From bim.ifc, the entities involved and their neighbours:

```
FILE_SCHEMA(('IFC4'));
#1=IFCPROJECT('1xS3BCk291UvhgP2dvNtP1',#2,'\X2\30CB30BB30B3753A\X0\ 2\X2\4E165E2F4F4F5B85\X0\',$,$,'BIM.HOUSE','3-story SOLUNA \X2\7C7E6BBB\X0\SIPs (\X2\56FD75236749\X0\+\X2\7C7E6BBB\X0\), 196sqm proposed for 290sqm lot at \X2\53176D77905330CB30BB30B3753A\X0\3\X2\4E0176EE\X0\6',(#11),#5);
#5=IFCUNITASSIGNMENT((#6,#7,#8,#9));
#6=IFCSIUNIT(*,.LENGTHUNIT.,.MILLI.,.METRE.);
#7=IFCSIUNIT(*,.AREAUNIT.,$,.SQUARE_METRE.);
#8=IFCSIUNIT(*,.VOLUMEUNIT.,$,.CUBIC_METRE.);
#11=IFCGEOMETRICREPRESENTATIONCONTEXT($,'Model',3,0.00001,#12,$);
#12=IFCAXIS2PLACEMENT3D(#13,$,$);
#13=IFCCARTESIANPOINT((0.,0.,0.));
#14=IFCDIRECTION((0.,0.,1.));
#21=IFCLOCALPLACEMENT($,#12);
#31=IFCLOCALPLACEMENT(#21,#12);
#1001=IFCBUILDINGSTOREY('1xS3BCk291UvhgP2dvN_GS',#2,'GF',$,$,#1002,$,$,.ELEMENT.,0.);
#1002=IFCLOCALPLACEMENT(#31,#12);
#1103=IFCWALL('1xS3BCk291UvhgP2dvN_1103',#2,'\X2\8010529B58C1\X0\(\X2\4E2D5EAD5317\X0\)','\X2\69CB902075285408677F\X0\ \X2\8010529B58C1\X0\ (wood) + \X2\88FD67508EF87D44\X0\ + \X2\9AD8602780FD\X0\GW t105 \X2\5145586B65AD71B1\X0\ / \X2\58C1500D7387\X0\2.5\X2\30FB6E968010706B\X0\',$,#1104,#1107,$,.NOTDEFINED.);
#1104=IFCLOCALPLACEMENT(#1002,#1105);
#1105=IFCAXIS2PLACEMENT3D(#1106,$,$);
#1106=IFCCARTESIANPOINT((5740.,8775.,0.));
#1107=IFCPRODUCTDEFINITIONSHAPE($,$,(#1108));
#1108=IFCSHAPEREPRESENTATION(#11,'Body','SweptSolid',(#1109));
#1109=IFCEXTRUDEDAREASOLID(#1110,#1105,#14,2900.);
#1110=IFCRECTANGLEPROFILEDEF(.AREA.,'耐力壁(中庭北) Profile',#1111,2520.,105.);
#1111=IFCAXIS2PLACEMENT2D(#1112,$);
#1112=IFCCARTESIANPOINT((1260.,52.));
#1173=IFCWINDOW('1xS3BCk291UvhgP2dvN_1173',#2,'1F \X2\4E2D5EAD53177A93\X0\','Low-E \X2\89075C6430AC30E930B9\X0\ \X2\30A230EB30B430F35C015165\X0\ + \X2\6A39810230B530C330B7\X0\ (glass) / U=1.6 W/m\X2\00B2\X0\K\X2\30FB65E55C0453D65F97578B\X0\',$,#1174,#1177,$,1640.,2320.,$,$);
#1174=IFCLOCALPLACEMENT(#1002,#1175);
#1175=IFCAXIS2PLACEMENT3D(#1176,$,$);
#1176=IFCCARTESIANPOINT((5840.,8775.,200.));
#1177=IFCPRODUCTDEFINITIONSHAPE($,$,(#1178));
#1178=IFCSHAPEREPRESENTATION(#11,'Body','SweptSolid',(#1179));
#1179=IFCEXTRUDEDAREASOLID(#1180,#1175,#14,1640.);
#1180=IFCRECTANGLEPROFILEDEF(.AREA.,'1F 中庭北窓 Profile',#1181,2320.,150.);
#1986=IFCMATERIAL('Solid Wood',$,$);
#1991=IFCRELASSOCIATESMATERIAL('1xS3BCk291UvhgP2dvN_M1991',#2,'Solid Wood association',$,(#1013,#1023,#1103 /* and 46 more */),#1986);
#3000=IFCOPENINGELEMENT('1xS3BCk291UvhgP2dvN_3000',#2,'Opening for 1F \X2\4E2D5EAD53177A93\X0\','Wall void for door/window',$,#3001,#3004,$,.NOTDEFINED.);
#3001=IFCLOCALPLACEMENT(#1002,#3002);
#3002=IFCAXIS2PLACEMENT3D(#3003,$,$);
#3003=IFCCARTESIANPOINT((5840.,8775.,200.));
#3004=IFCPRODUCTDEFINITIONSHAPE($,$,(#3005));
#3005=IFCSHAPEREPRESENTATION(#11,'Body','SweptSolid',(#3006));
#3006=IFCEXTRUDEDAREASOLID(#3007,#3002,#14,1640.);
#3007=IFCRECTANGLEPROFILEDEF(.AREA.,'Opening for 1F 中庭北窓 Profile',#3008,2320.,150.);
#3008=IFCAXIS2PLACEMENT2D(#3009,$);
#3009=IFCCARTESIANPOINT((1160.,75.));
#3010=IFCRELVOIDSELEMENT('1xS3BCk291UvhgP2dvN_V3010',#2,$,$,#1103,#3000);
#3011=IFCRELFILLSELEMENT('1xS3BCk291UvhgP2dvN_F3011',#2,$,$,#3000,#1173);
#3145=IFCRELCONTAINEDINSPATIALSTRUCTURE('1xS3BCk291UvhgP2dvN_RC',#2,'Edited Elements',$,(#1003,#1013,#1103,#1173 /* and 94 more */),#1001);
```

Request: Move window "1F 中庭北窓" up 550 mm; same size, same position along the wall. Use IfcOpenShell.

```python
import numpy as np
import ifcopenshell
import ifcopenshell.api.geometry
import ifcopenshell.util.placement
import ifcopenshell.util.unit

model = ifcopenshell.open("bim.ifc")
unit_scale = ifcopenshell.util.unit.calculate_unit_scale(model)

window = model.by_guid("1xS3BCk291UvhgP2dvN_1173")
opening = window.FillsVoids[0].RelatingOpeningElement
dz = 550.0

shift = np.array([0.0, 0.0, dz])
# The window is not placed relative to its opening, so move both.
for product in (opening, window):
    matrix = ifcopenshell.util.placement.get_local_placement(product.ObjectPlacement)
    matrix[:3, 3] += shift
    ifcopenshell.api.geometry.edit_object_placement(model, product=product, matrix=matrix, is_si=False)

print(f"moved by {dz * unit_scale:+.3f} m")

model.write("bim-out.ifc")
```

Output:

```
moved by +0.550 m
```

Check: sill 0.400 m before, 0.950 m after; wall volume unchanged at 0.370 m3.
